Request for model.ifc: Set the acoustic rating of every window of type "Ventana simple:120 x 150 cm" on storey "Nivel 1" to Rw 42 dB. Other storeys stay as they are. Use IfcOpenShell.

First a look at what the model holds.

```python
import ifcopenshell
import ifcopenshell.util.element

model = ifcopenshell.open("model.ifc")
print(model.schema)
storey = next(s for s in model.by_type("IfcBuildingStorey") if s.Name == "Nivel 1")
windows = [e for e in ifcopenshell.util.element.get_decomposition(storey) if e.is_a("IfcWindow")]
seen = {}
for e in windows:
    element_type = ifcopenshell.util.element.get_type(e)
    key = (element_type.Name if element_type != e and element_type else None, ifcopenshell.util.element.get_pset(e, "Pset_WindowCommon", "AcousticRating"))
    seen[key] = seen.get(key, 0) + 1
for (name, value), count in sorted(seen.items(), key=str):
    print(count, "x", name, "|", value)
```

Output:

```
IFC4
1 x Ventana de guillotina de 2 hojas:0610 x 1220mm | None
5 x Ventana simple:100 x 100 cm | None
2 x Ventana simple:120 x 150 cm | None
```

```python
import ifcopenshell
import ifcopenshell.api.pset
import ifcopenshell.util.element

model = ifcopenshell.open("model.ifc")

storey = next(s for s in model.by_type("IfcBuildingStorey") if s.Name == "Nivel 1")
windows = [e for e in ifcopenshell.util.element.get_decomposition(storey) if e.is_a("IfcWindow")]

count = 0
for e in windows:
    element_type = ifcopenshell.util.element.get_type(e)
    if element_type in (None, e) or element_type.Name != "Ventana simple:120 x 150 cm":
        continue
    # add_pset returns the element's existing set when there is one.
    pset = ifcopenshell.api.pset.add_pset(model, product=e, name="Pset_WindowCommon")
    ifcopenshell.api.pset.edit_pset(model, pset=pset, properties={"AcousticRating": "Rw 42 dB"})
    count += 1

print(count, "windows updated")

model.write("model_updated.ifc")
```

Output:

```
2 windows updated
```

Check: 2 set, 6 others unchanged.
